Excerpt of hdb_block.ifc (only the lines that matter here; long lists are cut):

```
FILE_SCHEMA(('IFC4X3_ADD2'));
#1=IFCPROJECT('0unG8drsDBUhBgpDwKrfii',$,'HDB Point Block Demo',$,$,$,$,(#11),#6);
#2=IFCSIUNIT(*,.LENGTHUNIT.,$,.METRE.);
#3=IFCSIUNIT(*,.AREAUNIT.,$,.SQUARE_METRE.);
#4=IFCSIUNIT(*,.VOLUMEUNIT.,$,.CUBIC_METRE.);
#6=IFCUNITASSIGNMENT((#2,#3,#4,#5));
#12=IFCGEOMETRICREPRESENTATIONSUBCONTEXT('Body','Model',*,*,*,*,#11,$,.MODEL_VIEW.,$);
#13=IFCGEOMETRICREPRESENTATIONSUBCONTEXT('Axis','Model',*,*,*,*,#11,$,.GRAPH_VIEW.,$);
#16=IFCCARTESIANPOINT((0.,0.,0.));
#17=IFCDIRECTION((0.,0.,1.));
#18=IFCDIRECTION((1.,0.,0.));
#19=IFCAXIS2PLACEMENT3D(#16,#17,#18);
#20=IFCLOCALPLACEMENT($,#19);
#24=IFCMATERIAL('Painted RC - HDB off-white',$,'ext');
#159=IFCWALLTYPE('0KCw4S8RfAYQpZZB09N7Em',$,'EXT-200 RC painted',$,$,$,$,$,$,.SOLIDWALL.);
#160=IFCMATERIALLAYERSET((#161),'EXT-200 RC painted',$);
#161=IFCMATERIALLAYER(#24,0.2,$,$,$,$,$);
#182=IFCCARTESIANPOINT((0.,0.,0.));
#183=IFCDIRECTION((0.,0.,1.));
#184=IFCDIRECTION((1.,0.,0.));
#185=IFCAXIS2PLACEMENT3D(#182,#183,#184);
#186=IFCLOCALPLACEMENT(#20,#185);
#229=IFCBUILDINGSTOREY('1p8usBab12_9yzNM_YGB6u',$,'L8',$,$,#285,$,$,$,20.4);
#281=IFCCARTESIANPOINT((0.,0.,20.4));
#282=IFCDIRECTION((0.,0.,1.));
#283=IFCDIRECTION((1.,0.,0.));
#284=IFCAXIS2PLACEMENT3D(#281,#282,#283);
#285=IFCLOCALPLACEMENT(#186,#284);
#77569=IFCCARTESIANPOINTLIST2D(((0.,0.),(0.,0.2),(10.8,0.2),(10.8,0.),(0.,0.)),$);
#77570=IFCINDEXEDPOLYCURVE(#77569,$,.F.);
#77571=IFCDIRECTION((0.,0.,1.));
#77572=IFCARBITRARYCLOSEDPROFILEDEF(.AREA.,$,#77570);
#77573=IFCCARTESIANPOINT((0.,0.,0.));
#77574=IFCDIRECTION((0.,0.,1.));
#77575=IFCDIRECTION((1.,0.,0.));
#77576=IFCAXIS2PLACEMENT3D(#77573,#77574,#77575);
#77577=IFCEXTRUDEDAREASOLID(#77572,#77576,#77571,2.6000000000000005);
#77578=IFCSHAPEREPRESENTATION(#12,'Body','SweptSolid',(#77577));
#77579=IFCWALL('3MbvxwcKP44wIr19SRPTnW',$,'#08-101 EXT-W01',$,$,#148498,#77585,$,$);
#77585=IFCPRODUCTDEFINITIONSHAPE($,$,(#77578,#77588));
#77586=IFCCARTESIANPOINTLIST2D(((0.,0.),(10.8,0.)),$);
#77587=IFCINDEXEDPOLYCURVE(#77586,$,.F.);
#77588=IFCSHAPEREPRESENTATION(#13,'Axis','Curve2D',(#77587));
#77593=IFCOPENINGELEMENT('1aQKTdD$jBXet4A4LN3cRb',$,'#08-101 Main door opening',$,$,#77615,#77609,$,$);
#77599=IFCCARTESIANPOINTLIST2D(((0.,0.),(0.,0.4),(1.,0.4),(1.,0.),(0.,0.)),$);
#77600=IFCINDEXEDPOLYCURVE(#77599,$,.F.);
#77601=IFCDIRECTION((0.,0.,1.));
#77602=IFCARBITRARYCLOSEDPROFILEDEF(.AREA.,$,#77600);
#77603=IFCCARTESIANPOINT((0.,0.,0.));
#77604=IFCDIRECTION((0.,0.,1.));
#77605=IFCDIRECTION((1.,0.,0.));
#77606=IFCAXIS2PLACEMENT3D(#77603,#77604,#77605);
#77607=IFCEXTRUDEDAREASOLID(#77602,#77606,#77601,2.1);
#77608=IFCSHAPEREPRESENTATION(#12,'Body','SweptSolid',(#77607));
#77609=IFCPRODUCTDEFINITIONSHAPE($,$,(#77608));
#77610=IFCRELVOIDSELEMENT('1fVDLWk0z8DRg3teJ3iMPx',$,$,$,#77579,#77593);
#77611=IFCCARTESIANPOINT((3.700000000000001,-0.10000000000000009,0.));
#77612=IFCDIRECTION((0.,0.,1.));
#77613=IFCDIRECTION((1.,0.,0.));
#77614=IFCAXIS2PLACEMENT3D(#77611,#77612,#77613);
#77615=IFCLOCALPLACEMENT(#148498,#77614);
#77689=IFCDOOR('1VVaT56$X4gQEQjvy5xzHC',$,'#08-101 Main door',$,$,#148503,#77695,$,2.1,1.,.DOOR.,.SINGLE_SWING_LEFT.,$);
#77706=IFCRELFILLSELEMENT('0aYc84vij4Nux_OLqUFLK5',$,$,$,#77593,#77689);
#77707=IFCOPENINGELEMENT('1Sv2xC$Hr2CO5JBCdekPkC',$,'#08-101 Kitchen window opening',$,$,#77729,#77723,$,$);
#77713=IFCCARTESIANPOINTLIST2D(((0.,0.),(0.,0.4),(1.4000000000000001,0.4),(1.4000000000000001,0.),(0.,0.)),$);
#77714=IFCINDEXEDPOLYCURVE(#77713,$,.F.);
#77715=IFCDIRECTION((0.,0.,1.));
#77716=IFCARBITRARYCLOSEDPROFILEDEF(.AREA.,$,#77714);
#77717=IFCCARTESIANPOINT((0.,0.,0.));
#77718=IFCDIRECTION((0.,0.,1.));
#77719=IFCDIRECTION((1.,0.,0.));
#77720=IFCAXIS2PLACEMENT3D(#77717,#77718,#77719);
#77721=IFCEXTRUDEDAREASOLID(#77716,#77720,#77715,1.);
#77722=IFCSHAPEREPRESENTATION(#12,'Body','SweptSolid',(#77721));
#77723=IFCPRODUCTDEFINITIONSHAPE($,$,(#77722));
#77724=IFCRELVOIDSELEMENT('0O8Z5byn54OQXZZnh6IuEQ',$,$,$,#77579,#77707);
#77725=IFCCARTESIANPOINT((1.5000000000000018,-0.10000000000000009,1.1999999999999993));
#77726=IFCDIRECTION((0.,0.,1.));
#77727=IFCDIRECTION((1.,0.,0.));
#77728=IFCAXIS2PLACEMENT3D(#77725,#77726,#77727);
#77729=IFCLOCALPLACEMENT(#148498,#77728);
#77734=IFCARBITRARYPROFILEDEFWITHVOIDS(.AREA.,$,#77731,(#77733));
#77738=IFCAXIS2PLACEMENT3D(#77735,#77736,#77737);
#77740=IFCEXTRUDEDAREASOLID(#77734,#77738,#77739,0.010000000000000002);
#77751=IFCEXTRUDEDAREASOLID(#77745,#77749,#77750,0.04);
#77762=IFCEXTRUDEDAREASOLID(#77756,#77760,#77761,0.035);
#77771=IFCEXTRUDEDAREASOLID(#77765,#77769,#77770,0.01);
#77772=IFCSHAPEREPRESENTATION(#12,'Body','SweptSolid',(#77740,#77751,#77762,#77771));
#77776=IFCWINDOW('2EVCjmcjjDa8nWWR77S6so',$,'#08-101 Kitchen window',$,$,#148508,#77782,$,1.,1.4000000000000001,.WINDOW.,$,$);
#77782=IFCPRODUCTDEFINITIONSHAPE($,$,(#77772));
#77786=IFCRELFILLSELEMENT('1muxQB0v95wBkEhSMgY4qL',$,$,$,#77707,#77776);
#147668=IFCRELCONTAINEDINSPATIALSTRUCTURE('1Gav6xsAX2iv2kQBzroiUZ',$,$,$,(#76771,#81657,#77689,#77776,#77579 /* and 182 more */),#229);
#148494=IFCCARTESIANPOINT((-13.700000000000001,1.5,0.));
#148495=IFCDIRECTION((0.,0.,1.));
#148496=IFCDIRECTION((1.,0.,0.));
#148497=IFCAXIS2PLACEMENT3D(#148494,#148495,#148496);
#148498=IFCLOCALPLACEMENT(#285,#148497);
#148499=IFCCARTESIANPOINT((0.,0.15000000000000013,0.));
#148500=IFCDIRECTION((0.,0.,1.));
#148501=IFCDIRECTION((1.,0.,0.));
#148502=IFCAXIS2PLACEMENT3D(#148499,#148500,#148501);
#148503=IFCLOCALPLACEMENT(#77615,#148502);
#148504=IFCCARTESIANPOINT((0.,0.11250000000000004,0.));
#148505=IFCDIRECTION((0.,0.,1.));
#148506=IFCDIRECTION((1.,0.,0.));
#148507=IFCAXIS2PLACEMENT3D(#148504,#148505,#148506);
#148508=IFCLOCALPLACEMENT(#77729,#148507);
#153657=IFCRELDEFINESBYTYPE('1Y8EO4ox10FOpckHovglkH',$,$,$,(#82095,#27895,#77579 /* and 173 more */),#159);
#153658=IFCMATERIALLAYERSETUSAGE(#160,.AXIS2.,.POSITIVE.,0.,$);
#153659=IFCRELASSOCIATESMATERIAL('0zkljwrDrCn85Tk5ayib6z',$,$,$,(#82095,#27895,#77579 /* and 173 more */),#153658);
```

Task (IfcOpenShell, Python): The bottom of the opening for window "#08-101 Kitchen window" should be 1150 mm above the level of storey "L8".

```python
import numpy as np
import ifcopenshell
import ifcopenshell.api.geometry
import ifcopenshell.geom
import ifcopenshell.util.element
import ifcopenshell.util.placement
import ifcopenshell.util.shape
import ifcopenshell.util.unit

model = ifcopenshell.open("hdb_block.ifc")
unit_scale = ifcopenshell.util.unit.calculate_unit_scale(model)

window = model.by_id(77776)
opening = window.FillsVoids[0].RelatingOpeningElement
storey = ifcopenshell.util.element.get_container(window, ifc_class="IfcBuildingStorey")
level = ifcopenshell.util.placement.get_local_placement(storey.ObjectPlacement)[2, 3]

# The opening's origin need not be at the sill, so measure its lowest point.
shape = ifcopenshell.geom.create_shape(ifcopenshell.geom.settings(), opening)
bottom = ifcopenshell.util.shape.get_shape_bottom_elevation(shape, shape.geometry) / unit_scale
dz = level + 1.15 / unit_scale - bottom

shift = np.array([0.0, 0.0, dz])
# The window is placed relative to its opening, so it follows when the opening moves.
matrix = ifcopenshell.util.placement.get_local_placement(opening.ObjectPlacement)
matrix[:3, 3] += shift
ifcopenshell.api.geometry.edit_object_placement(
    model, product=opening, matrix=matrix, is_si=False, should_transform_children=True
)

print(f"moved by {dz * unit_scale:+.3f} m")

model.write("hdb_block-out.ifc")
```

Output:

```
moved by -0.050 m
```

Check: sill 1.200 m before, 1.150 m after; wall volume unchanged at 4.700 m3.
